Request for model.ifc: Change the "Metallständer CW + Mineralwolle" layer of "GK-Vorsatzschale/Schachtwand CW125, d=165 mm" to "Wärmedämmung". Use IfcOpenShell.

First a look at what the model holds.

```python
import ifcopenshell
import ifcopenshell.util.element

model = ifcopenshell.open("model.ifc")
print(model.schema)
for layer_set in model.by_type("IfcMaterialLayerSet"):
    if layer_set.LayerSetName == "GK-Vorsatzschale/Schachtwand CW125, d=165 mm":
        for layer in layer_set.MaterialLayers:
            print(layer.id(), layer.Material and layer.Material.Name, layer.LayerThickness, sep=" | ")
        print(len(ifcopenshell.util.element.get_elements_by_material(model, layer_set)), "elements and types use it")
print(sorted(m.Name for m in model.by_type("IfcMaterial") if m.Name)[:60])
```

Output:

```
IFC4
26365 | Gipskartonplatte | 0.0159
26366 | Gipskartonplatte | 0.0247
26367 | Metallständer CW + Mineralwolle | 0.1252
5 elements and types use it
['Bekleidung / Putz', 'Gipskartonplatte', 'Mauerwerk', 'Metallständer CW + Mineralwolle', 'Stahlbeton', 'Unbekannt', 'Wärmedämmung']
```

```python
import ifcopenshell
import ifcopenshell.api.material

model = ifcopenshell.open("model.ifc")

layer_set = next(s for s in model.by_type("IfcMaterialLayerSet") if s.LayerSetName == "GK-Vorsatzschale/Schachtwand CW125, d=165 mm")
layer = next(l for l in layer_set.MaterialLayers if l.Material and l.Material.Name == "Metallständer CW + Mineralwolle")
material = next(m for m in model.by_type("IfcMaterial") if m.Name == "Wärmedämmung")

# Point this one layer at the other material; renaming the old one would change it everywhere.
ifcopenshell.api.material.edit_layer(model, layer=layer, attributes={"Name": material.Name}, material=material)

print([l.Material.Name if l.Material else None for l in layer_set.MaterialLayers])

model.write("model_updated.ifc")
```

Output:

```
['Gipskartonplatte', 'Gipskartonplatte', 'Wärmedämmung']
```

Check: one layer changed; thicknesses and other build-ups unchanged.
